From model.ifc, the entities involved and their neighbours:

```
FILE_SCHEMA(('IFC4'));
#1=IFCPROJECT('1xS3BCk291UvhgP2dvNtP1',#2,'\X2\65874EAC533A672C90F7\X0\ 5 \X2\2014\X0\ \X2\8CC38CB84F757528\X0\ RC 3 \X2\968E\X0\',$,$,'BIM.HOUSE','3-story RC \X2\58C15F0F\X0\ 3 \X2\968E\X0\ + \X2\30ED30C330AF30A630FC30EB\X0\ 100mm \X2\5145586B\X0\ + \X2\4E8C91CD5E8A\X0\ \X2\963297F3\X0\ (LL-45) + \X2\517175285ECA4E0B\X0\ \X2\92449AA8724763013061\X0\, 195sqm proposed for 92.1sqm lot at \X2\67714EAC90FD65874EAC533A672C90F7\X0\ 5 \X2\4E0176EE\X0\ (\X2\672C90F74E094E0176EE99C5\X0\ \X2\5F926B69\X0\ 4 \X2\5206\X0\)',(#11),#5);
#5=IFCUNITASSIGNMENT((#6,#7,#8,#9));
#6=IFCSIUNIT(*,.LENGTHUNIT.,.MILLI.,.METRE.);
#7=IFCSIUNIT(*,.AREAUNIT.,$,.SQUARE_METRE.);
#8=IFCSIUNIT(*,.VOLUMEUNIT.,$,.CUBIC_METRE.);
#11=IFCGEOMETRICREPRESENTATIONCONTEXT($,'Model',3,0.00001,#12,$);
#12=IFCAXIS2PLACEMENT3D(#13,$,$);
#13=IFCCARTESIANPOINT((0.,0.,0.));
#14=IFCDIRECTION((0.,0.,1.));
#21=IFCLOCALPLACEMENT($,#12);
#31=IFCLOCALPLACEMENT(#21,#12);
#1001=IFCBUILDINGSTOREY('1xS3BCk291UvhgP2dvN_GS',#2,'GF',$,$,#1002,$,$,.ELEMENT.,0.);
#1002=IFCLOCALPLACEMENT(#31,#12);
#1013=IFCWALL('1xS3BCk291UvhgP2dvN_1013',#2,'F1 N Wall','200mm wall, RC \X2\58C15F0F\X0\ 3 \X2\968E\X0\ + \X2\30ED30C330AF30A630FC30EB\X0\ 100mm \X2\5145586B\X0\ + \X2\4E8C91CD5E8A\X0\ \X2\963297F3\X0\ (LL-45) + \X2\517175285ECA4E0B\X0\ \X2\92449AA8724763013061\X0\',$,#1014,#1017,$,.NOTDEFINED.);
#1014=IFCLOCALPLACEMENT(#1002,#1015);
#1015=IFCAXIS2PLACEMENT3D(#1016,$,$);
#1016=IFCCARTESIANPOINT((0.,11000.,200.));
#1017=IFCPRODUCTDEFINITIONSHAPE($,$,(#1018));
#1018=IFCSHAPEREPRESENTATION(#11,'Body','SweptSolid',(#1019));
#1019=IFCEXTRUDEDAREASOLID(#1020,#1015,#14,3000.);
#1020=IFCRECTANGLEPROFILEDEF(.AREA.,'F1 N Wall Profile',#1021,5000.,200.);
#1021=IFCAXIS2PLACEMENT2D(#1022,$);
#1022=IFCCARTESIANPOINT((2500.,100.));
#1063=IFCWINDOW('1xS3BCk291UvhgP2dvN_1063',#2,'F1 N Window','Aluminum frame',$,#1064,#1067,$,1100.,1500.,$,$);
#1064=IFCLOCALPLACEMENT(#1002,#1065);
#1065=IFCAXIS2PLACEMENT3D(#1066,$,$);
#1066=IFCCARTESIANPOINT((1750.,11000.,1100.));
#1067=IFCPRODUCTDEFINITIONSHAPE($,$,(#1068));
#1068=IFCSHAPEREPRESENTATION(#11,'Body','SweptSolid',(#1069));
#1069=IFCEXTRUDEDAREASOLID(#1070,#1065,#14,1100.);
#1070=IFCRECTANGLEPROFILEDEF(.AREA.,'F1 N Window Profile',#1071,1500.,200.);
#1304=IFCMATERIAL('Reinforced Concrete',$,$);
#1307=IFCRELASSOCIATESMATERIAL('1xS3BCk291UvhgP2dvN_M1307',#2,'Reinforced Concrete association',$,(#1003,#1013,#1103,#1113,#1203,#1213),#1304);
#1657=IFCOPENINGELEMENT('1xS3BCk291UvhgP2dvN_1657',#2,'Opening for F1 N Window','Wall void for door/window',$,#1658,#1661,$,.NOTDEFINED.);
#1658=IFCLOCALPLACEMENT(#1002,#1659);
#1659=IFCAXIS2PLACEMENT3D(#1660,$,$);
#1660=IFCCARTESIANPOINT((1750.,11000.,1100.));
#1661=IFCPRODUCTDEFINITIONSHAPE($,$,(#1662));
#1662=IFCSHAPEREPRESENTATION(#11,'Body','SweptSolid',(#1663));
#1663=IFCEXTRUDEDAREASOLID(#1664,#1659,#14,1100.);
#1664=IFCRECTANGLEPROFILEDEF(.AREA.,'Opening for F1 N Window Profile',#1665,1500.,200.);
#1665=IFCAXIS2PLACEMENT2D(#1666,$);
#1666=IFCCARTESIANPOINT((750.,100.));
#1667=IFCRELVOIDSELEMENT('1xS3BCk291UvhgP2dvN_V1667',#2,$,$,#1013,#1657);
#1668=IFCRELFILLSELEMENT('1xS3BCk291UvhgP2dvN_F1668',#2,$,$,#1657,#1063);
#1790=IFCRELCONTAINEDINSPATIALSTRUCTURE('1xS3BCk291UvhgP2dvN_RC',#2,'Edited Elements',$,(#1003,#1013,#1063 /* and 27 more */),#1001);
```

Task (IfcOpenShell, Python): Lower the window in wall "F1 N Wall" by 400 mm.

```python
import numpy as np
import ifcopenshell
import ifcopenshell.api.geometry
import ifcopenshell.util.placement
import ifcopenshell.util.unit

model = ifcopenshell.open("model.ifc")
unit_scale = ifcopenshell.util.unit.calculate_unit_scale(model)

window = model.by_guid("1xS3BCk291UvhgP2dvN_1063")
opening = window.FillsVoids[0].RelatingOpeningElement
dz = -0.4 / unit_scale

shift = np.array([0.0, 0.0, dz])
# The window is not placed relative to its opening, so move both.
for product in (opening, window):
    matrix = ifcopenshell.util.placement.get_local_placement(product.ObjectPlacement)
    matrix[:3, 3] += shift
    ifcopenshell.api.geometry.edit_object_placement(model, product=product, matrix=matrix, is_si=False)

print(f"moved by {dz * unit_scale:+.3f} m")

model.write("model_v2.ifc")
```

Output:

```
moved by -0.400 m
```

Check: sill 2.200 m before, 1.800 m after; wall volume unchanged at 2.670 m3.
